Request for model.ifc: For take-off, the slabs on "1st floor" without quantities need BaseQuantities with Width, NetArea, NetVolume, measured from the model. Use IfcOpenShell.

First a look at what the model holds.

```python
import ifcopenshell
import ifcopenshell.util.element
import ifcopenshell.util.unit

model = ifcopenshell.open("model.ifc")
print(model.schema)
for unit_type in ("LENGTHUNIT", "AREAUNIT", "VOLUMEUNIT"):
    print(unit_type, ifcopenshell.util.unit.calculate_unit_scale(model, unit_type))
storey = next(s for s in model.by_type("IfcBuildingStorey") if s.Name == "1st floor")
slabs = [e for e in ifcopenshell.util.element.get_decomposition(storey) if e.is_a("IfcSlab")]
for e in sorted(slabs, key=lambda e: e.id()):
    print(e.id(), e.is_a(), e.Name, list(ifcopenshell.util.element.get_psets(e, qtos_only=True)), sep=" | ")
```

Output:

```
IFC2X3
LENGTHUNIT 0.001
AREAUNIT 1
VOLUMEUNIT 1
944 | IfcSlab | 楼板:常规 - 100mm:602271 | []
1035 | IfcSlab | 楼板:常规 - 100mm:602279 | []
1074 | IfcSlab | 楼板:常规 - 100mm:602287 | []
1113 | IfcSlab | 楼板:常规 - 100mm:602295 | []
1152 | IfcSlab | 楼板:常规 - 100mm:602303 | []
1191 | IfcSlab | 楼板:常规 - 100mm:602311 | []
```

```python
import ifcopenshell
import ifcopenshell.api.pset
import ifcopenshell.geom
import ifcopenshell.util.element
import ifcopenshell.util.shape
import ifcopenshell.util.unit

model = ifcopenshell.open("model.ifc")
unit_scale = ifcopenshell.util.unit.calculate_unit_scale(model)
area_scale = ifcopenshell.util.unit.calculate_unit_scale(model, "AREAUNIT")
volume_scale = ifcopenshell.util.unit.calculate_unit_scale(model, "VOLUMEUNIT")
settings = ifcopenshell.geom.settings()

storey = next(s for s in model.by_type("IfcBuildingStorey") if s.Name == "1st floor")
slabs = [e for e in ifcopenshell.util.element.get_decomposition(storey) if e.is_a("IfcSlab")]

for e in sorted(slabs, key=lambda e: e.id()):
    if ifcopenshell.util.element.get_psets(e, qtos_only=True, should_inherit=False):
        continue
    # Geometry comes back in metres, in the element's own axes.
    shape = ifcopenshell.geom.create_shape(settings, e)
    values = {
        "Width": ifcopenshell.util.shape.get_z(shape.geometry) / unit_scale,
        "NetArea": ifcopenshell.util.shape.get_footprint_area(shape.geometry) / area_scale,
        "NetVolume": ifcopenshell.util.shape.get_volume(shape.geometry) / volume_scale,
    }
    qto = ifcopenshell.api.pset.add_qto(model, product=e, name="BaseQuantities")
    ifcopenshell.api.pset.edit_qto(model, qto=qto, properties=values)
    print(e.id(), {k: round(v, 3) for k, v in values.items()})

model.write("model-out.ifc")
```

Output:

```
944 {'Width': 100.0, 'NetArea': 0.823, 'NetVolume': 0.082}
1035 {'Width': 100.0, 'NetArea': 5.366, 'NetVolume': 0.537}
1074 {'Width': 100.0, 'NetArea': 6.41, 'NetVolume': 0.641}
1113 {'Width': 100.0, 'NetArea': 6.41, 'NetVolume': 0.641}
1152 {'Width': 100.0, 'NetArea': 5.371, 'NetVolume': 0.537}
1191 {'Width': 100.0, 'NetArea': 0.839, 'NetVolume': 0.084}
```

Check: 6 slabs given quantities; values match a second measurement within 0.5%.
